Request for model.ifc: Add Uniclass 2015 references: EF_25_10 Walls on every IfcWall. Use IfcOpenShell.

First a look at what the model holds.

```python
import ifcopenshell

model = ifcopenshell.open("model.ifc")
print(model.schema)
print("classifications:", [c.Name for c in model.by_type("IfcClassification")])
for ifc_class in ("IfcDoor", "IfcRoof", "IfcStair", "IfcWall", "IfcWindow"):
    print(ifc_class, len(model.by_type(ifc_class)))
```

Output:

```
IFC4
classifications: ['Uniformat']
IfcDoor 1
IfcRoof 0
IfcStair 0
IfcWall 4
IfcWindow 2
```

```python
import ifcopenshell
import ifcopenshell.api.classification

model = ifcopenshell.open("model.ifc")

system = ifcopenshell.api.classification.add_classification(model, classification="Uniclass 2015")

codes = {
    "IfcWall": ("EF_25_10", "Walls"),
}
for ifc_class, (code, name) in codes.items():
    products = model.by_type(ifc_class)
    ifcopenshell.api.classification.add_reference(
        model, products=products, classification=system, identification=code, name=name
    )
    print(code, len(products))

model.write("model_rev.ifc")
```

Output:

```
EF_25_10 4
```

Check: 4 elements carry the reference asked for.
